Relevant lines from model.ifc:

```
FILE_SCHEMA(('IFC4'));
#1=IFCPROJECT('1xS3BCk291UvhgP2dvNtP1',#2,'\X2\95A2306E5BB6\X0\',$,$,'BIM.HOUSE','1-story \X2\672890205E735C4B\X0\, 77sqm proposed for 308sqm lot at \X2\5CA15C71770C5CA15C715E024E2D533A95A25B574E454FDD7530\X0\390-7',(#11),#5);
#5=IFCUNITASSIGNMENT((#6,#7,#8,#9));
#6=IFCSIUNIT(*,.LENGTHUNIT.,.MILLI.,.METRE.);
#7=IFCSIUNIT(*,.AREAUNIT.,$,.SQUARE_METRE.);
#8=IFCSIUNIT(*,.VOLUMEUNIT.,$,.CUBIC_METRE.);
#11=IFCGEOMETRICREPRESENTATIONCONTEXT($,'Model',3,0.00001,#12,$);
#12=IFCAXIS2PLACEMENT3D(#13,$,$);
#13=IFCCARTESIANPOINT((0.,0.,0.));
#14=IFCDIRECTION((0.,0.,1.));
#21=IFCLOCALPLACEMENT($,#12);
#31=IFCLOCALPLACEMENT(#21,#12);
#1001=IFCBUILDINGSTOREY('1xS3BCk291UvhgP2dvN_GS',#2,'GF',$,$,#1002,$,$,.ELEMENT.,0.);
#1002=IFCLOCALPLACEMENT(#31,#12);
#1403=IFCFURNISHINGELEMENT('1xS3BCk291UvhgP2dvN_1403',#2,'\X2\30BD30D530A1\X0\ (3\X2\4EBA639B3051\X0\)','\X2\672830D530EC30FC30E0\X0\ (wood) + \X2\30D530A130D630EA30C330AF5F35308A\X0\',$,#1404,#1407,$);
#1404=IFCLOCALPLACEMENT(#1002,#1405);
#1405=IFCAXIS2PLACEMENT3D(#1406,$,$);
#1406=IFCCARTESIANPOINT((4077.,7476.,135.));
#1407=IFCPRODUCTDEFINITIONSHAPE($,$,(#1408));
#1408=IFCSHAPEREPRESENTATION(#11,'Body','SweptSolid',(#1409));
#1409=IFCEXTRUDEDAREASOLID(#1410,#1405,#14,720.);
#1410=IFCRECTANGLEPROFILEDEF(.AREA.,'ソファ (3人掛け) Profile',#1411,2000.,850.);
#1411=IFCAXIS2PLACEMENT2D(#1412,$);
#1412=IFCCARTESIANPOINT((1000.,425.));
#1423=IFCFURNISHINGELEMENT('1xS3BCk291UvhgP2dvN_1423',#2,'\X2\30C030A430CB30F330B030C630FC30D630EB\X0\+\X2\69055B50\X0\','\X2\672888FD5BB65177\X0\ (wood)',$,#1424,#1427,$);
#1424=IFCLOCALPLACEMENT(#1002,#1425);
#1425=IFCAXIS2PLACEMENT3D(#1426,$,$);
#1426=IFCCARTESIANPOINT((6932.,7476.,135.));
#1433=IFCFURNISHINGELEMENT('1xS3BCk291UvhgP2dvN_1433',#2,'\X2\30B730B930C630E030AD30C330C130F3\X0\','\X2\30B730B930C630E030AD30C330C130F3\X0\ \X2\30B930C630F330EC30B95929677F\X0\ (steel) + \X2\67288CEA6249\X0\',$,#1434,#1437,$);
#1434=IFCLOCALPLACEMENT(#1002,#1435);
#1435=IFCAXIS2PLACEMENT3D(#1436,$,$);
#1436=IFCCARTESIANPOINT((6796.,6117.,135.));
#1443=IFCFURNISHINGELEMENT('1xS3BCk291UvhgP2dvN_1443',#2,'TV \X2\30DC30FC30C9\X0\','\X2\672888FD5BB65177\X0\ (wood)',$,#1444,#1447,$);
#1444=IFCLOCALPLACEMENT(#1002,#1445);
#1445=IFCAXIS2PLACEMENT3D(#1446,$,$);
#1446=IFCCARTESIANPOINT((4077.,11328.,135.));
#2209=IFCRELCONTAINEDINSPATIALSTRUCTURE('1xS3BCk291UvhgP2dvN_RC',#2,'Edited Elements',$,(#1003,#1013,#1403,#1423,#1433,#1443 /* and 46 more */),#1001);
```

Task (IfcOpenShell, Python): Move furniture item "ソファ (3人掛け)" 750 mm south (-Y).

```python
import ifcopenshell
import ifcopenshell.api.geometry
import ifcopenshell.util.placement

model = ifcopenshell.open("model.ifc")

item = model.by_guid("1xS3BCk291UvhgP2dvN_1403")
matrix = ifcopenshell.util.placement.get_local_placement(item.ObjectPlacement)
matrix[1, 3] -= 750.0
ifcopenshell.api.geometry.edit_object_placement(model, product=item, matrix=matrix, is_si=False)

print(ifcopenshell.util.placement.get_local_placement(item.ObjectPlacement).round(3) + 0.0)

model.write("model-out.ifc")
```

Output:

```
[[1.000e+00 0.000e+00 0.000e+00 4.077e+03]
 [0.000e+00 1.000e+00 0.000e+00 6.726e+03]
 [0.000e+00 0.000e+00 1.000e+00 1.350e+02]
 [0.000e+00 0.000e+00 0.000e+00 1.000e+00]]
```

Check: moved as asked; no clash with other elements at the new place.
